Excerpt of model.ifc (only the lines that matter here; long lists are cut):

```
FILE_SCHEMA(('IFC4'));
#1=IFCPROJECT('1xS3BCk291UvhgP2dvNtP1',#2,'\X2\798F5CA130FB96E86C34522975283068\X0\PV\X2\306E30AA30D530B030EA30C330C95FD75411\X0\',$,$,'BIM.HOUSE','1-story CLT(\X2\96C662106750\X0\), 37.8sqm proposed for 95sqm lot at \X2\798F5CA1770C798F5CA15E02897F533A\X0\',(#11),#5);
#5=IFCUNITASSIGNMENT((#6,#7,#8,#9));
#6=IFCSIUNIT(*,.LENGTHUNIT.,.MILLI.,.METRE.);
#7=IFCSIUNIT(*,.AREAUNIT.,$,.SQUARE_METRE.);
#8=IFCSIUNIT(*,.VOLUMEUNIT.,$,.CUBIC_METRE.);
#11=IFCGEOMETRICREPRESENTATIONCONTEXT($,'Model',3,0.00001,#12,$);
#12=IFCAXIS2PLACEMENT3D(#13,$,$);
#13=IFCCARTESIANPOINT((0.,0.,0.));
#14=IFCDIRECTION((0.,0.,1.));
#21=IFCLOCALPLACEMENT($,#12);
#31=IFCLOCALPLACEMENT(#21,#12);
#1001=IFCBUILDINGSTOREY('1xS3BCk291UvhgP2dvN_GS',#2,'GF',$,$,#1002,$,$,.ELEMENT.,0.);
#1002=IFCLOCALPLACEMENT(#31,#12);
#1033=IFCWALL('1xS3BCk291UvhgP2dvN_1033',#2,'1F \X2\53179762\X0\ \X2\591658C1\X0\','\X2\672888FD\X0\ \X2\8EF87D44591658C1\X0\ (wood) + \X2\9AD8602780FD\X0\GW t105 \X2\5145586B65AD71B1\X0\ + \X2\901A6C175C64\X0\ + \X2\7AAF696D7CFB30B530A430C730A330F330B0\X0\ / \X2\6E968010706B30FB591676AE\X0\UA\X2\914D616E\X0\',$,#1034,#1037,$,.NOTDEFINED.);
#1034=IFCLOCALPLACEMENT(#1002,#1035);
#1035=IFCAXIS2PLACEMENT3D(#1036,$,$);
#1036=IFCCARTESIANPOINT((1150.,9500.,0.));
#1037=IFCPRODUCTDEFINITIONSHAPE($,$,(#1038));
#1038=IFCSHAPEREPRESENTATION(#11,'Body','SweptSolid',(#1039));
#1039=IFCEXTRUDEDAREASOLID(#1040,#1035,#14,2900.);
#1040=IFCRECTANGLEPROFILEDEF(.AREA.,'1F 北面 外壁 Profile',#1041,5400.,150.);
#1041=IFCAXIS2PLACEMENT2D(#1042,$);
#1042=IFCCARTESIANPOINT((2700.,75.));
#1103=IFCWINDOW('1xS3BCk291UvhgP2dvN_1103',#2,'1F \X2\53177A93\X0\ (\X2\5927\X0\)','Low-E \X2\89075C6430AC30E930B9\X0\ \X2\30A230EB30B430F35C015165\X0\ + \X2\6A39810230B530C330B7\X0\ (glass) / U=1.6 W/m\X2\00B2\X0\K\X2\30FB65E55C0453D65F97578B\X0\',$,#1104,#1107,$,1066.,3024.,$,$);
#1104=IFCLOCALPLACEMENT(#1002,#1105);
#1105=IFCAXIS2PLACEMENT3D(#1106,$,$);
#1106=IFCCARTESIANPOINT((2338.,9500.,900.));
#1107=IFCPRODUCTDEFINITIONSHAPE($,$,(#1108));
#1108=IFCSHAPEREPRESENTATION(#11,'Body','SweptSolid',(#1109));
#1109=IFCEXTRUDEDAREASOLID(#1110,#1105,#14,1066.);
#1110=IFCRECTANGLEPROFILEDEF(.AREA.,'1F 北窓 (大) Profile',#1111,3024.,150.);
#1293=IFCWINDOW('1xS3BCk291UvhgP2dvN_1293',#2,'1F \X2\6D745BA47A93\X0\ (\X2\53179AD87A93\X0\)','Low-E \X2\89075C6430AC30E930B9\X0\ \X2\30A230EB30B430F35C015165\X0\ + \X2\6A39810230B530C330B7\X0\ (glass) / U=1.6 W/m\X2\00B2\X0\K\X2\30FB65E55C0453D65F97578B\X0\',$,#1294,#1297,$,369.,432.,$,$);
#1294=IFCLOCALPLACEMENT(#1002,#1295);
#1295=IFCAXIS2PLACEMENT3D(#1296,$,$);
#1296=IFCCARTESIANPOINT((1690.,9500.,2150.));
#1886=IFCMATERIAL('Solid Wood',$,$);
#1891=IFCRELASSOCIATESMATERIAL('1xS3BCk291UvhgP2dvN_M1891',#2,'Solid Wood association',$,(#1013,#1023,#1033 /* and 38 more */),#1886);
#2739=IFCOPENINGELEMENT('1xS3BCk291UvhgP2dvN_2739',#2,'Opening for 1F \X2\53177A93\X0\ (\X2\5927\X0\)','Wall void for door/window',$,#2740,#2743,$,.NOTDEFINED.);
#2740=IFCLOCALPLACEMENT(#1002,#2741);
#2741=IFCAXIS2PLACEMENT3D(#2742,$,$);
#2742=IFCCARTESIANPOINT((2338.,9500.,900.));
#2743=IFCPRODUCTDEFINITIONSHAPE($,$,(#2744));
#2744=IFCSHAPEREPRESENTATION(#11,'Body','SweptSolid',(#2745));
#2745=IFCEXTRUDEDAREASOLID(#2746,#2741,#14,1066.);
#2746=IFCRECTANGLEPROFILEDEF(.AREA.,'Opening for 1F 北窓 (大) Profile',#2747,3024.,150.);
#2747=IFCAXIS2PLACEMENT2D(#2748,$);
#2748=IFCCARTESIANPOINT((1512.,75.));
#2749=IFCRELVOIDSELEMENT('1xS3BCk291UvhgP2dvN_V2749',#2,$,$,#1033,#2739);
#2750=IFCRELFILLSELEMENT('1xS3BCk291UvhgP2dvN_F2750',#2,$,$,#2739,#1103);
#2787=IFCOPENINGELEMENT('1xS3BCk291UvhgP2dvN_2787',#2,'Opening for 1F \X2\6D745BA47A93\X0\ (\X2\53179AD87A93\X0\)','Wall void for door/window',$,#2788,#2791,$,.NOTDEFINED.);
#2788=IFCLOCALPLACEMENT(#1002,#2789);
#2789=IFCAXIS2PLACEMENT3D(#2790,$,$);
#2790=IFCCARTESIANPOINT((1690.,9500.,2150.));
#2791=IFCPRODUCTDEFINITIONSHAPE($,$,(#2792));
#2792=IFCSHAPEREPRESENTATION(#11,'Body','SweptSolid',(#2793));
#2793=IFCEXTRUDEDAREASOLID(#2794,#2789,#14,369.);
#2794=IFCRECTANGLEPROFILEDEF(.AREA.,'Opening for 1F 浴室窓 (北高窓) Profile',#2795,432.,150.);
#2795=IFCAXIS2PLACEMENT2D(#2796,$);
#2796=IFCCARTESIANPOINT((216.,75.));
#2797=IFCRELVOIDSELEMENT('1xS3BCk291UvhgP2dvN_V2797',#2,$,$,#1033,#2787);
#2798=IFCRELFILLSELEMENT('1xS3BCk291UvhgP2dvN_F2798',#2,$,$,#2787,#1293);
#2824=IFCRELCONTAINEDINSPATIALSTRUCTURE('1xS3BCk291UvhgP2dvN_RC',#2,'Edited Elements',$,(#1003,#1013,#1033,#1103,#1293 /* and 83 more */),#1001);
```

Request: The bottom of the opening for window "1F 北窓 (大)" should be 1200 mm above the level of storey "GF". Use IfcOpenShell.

```python
import numpy as np
import ifcopenshell
import ifcopenshell.api.geometry
import ifcopenshell.geom
import ifcopenshell.util.element
import ifcopenshell.util.placement
import ifcopenshell.util.shape
import ifcopenshell.util.unit

model = ifcopenshell.open("model.ifc")
unit_scale = ifcopenshell.util.unit.calculate_unit_scale(model)

window = model.by_id(1103)
opening = window.FillsVoids[0].RelatingOpeningElement
storey = ifcopenshell.util.element.get_container(window, ifc_class="IfcBuildingStorey")
level = ifcopenshell.util.placement.get_local_placement(storey.ObjectPlacement)[2, 3]

# The opening's origin need not be at the sill, so measure its lowest point.
shape = ifcopenshell.geom.create_shape(ifcopenshell.geom.settings(), opening)
bottom = ifcopenshell.util.shape.get_shape_bottom_elevation(shape, shape.geometry) / unit_scale
dz = level + 1.2 / unit_scale - bottom

shift = np.array([0.0, 0.0, dz])
# The window is not placed relative to its opening, so move both.
for product in (opening, window):
    matrix = ifcopenshell.util.placement.get_local_placement(product.ObjectPlacement)
    matrix[:3, 3] += shift
    ifcopenshell.api.geometry.edit_object_placement(model, product=product, matrix=matrix, is_si=False)

print(f"moved by {dz * unit_scale:+.3f} m")

model.write("model-out.ifc")
```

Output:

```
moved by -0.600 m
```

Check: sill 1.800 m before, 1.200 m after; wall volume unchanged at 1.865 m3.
